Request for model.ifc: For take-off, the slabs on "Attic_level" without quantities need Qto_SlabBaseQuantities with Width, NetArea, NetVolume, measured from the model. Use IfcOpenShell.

First a look at what the model holds.

```python
import ifcopenshell
import ifcopenshell.util.element
import ifcopenshell.util.unit

model = ifcopenshell.open("model.ifc")
print(model.schema)
for unit_type in ("LENGTHUNIT", "AREAUNIT", "VOLUMEUNIT"):
    print(unit_type, ifcopenshell.util.unit.calculate_unit_scale(model, unit_type))
storey = next(s for s in model.by_type("IfcBuildingStorey") if s.Name == "Attic_level")
slabs = [e for e in ifcopenshell.util.element.get_decomposition(storey) if e.is_a("IfcSlab")]
for e in sorted(slabs, key=lambda e: e.id()):
    print(e.id(), e.is_a(), e.Name, list(ifcopenshell.util.element.get_psets(e, qtos_only=True)), sep=" | ")
```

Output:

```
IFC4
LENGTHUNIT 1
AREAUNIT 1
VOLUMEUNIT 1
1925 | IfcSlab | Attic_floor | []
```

```python
import ifcopenshell
import ifcopenshell.api.pset
import ifcopenshell.geom
import ifcopenshell.util.element
import ifcopenshell.util.shape
import ifcopenshell.util.unit

model = ifcopenshell.open("model.ifc")
unit_scale = ifcopenshell.util.unit.calculate_unit_scale(model)
area_scale = ifcopenshell.util.unit.calculate_unit_scale(model, "AREAUNIT")
volume_scale = ifcopenshell.util.unit.calculate_unit_scale(model, "VOLUMEUNIT")
settings = ifcopenshell.geom.settings()

storey = next(s for s in model.by_type("IfcBuildingStorey") if s.Name == "Attic_level")
slabs = [e for e in ifcopenshell.util.element.get_decomposition(storey) if e.is_a("IfcSlab")]

for e in sorted(slabs, key=lambda e: e.id()):
    if ifcopenshell.util.element.get_psets(e, qtos_only=True, should_inherit=False):
        continue
    # Geometry comes back in metres, in the element's own axes.
    shape = ifcopenshell.geom.create_shape(settings, e)
    values = {
        "Width": ifcopenshell.util.shape.get_z(shape.geometry) / unit_scale,
        "NetArea": ifcopenshell.util.shape.get_footprint_area(shape.geometry) / area_scale,
        "NetVolume": ifcopenshell.util.shape.get_volume(shape.geometry) / volume_scale,
    }
    qto = ifcopenshell.api.pset.add_qto(model, product=e, name="Qto_SlabBaseQuantities")
    ifcopenshell.api.pset.edit_qto(model, qto=qto, properties=values)
    print(e.id(), {k: round(v, 3) for k, v in values.items()})

model.write("model_rev.ifc")
```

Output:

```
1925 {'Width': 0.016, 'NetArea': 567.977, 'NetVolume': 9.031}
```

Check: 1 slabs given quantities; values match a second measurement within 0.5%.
